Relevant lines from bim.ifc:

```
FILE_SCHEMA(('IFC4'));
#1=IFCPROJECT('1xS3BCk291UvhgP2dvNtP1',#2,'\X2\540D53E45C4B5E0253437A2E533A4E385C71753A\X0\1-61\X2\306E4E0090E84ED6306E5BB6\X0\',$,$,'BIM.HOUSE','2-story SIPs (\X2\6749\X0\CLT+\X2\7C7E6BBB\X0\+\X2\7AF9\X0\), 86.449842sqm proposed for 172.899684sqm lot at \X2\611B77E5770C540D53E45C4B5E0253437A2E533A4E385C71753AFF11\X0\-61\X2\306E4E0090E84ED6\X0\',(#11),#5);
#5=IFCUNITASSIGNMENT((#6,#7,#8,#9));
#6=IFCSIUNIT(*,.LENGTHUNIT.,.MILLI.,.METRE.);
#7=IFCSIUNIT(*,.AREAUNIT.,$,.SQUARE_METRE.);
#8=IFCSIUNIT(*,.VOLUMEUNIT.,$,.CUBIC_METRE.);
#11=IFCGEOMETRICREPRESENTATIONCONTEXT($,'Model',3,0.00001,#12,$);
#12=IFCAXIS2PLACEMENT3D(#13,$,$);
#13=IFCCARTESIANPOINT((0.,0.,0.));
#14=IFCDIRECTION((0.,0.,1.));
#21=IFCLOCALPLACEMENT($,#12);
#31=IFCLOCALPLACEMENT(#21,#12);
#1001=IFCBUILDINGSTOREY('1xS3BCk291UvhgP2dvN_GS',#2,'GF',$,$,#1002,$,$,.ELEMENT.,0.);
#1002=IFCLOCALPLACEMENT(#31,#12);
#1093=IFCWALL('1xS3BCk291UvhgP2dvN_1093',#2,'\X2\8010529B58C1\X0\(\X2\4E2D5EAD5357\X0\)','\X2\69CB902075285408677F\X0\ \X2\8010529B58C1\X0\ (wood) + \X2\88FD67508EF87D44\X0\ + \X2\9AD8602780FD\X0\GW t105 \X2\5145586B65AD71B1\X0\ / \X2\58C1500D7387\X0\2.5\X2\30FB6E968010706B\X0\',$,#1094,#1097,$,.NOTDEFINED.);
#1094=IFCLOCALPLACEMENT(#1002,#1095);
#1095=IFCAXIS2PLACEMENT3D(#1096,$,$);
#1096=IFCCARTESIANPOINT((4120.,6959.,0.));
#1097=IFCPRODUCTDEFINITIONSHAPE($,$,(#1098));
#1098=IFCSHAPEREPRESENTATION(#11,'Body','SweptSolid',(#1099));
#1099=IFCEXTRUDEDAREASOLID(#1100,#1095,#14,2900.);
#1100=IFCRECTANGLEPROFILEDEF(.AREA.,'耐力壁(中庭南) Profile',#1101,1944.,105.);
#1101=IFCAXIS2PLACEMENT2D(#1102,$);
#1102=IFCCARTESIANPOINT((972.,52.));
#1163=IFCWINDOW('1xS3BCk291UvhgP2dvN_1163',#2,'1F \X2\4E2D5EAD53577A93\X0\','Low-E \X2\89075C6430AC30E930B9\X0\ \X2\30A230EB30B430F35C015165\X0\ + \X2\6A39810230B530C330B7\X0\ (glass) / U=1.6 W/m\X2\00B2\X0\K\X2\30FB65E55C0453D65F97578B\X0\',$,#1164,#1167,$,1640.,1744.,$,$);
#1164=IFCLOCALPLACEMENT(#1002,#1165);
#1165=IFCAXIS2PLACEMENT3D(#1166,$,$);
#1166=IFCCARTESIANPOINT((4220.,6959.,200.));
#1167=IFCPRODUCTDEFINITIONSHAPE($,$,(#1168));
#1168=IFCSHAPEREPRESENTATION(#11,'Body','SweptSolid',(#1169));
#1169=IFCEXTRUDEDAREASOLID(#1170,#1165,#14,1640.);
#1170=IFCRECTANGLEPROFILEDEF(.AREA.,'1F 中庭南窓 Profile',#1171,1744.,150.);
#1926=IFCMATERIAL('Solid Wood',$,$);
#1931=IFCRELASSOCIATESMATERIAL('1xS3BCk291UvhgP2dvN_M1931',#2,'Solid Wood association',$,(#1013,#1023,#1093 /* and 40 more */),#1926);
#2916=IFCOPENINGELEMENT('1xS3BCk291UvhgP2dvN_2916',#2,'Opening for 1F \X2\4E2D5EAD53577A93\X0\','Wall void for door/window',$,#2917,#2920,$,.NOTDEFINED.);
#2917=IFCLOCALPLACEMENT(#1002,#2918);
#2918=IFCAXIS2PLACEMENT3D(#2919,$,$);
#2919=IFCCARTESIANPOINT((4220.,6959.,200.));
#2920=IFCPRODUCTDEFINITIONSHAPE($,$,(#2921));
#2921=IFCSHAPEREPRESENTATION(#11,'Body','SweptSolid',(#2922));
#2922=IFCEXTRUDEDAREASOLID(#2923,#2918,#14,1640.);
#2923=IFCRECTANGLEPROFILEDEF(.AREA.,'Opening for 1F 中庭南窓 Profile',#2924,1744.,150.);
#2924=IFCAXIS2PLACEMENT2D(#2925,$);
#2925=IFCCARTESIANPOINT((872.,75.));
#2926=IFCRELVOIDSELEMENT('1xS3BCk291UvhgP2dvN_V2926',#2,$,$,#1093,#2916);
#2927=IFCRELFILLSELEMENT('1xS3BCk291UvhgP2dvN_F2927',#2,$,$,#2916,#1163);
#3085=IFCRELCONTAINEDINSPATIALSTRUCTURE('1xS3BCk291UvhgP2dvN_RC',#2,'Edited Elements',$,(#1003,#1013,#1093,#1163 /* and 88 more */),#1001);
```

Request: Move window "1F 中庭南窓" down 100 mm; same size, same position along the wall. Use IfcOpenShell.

```python
import numpy as np
import ifcopenshell
import ifcopenshell.api.geometry
import ifcopenshell.util.placement
import ifcopenshell.util.unit

model = ifcopenshell.open("bim.ifc")
unit_scale = ifcopenshell.util.unit.calculate_unit_scale(model)

window = model.by_guid("1xS3BCk291UvhgP2dvN_1163")
opening = window.FillsVoids[0].RelatingOpeningElement
dz = -0.1 / unit_scale

shift = np.array([0.0, 0.0, dz])
# The window is not placed relative to its opening, so move both.
for product in (opening, window):
    matrix = ifcopenshell.util.placement.get_local_placement(product.ObjectPlacement)
    matrix[:3, 3] += shift
    ifcopenshell.api.geometry.edit_object_placement(model, product=product, matrix=matrix, is_si=False)

print(f"moved by {dz * unit_scale:+.3f} m")

model.write("bim_updated.ifc")
```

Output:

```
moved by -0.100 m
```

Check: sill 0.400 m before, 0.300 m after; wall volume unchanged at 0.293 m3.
